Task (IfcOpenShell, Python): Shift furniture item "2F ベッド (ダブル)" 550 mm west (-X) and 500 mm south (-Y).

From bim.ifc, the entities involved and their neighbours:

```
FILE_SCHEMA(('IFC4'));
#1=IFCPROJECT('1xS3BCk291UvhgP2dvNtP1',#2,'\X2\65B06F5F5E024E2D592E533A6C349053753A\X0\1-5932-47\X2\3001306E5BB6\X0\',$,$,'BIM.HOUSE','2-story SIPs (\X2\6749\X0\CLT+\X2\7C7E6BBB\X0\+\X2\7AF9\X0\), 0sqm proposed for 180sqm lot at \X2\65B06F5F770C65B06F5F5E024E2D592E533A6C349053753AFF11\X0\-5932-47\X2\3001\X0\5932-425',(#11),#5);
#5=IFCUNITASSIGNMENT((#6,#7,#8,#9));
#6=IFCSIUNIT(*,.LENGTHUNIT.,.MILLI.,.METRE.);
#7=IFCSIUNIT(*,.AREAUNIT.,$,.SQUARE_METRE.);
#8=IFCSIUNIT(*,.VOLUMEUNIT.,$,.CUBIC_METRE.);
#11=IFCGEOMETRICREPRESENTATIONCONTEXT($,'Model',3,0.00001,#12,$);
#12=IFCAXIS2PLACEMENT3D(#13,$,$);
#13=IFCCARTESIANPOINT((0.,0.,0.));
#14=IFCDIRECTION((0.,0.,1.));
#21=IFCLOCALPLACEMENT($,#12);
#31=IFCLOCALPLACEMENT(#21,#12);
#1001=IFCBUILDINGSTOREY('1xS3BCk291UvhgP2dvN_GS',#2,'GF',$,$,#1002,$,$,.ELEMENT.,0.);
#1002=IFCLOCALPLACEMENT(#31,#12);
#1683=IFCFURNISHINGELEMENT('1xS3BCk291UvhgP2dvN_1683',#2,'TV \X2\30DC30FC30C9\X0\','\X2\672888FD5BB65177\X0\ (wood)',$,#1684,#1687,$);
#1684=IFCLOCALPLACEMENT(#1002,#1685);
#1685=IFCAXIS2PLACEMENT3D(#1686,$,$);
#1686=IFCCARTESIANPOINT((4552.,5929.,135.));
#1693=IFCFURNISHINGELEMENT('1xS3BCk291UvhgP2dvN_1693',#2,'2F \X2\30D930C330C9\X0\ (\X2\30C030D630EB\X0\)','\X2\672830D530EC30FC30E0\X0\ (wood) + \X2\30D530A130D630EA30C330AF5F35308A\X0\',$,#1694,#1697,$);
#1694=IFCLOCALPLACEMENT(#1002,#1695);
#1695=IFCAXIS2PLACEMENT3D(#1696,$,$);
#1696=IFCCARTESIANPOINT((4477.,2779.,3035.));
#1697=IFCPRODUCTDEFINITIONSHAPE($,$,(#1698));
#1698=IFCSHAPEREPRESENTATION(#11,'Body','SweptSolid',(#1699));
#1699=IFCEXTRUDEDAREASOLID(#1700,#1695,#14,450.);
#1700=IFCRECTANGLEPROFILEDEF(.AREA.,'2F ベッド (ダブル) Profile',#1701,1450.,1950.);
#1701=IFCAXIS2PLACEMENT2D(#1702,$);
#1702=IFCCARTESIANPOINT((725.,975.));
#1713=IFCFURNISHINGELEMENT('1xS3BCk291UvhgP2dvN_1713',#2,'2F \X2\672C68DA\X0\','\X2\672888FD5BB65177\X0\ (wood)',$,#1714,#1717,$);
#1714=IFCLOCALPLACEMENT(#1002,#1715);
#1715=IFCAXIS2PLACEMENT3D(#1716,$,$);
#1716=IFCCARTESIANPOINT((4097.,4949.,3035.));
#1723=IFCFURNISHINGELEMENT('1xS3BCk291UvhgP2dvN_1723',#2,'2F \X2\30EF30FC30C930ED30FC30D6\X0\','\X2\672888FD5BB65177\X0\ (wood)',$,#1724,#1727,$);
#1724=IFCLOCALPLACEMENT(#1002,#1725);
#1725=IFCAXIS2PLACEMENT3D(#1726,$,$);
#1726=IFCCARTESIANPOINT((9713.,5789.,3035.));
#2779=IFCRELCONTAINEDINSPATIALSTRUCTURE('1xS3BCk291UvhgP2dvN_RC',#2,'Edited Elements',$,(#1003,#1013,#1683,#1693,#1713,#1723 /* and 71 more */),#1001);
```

```python
import ifcopenshell
import ifcopenshell.api.geometry
import ifcopenshell.util.placement
import ifcopenshell.util.unit

model = ifcopenshell.open("bim.ifc")
unit_scale = ifcopenshell.util.unit.calculate_unit_scale(model)

item = model.by_guid("1xS3BCk291UvhgP2dvN_1693")
matrix = ifcopenshell.util.placement.get_local_placement(item.ObjectPlacement)
matrix[0, 3] -= 0.55 / unit_scale
matrix[1, 3] -= 0.5 / unit_scale
ifcopenshell.api.geometry.edit_object_placement(model, product=item, matrix=matrix, is_si=False)

print(ifcopenshell.util.placement.get_local_placement(item.ObjectPlacement).round(3) + 0.0)

model.write("bim_rev.ifc")
```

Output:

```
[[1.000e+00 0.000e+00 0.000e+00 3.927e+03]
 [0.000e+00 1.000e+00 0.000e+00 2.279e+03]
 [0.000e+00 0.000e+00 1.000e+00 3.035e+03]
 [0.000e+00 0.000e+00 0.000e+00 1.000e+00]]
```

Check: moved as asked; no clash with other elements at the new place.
